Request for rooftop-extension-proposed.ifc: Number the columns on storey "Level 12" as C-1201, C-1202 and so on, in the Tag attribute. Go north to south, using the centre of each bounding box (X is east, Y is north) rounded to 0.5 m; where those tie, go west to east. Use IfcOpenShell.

First a look at what the model holds.

```python
import ifcopenshell
import ifcopenshell.util.element
import ifcopenshell.util.placement

model = ifcopenshell.open("rooftop-extension-proposed.ifc")
print(model.schema)
storey = next(s for s in model.by_type("IfcBuildingStorey") if s.Name == "Level 12")
columns = [e for e in ifcopenshell.util.element.get_decomposition(storey) if e.is_a("IfcColumn")]
for e in sorted(columns, key=lambda e: e.id()):
    origin = ifcopenshell.util.placement.get_local_placement(e.ObjectPlacement)[:3, 3]
    print(e.id(), e.Tag, e.Name, origin.round(2) + 0.0, sep=" | ")
```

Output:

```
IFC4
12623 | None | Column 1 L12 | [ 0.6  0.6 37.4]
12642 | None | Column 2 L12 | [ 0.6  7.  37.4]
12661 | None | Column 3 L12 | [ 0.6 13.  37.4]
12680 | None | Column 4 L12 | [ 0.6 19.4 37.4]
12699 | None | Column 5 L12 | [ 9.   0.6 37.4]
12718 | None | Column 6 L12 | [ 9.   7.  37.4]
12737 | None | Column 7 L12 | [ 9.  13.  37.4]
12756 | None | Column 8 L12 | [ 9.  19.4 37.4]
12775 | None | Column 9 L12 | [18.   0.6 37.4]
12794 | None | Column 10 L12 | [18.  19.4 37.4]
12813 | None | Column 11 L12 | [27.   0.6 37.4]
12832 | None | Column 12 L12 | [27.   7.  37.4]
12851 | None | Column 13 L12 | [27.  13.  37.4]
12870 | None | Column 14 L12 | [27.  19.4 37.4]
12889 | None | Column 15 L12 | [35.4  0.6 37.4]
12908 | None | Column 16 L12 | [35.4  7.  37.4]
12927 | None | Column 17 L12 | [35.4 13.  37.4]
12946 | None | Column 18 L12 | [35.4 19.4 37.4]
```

```python
import ifcopenshell
import ifcopenshell.geom
import ifcopenshell.util.element
import ifcopenshell.util.shape

model = ifcopenshell.open("rooftop-extension-proposed.ifc")
settings = ifcopenshell.geom.settings()
settings.set("use-world-coords", True)


def centre(element):
    shape = ifcopenshell.geom.create_shape(settings, element)
    return ifcopenshell.util.shape.get_bbox_centroid(shape.geometry)


storey = next(s for s in model.by_type("IfcBuildingStorey") if s.Name == "Level 12")
columns = [e for e in ifcopenshell.util.element.get_decomposition(storey) if e.is_a("IfcColumn")]

# Insertion points can sit at a corner or the storey origin, so sort by the geometry (in metres).
centres = {e: centre(e) for e in columns}
columns.sort(key=lambda e: (-round(centres[e][1] / 0.5), centres[e][0]))

for i, e in enumerate(columns, start=1):
    number = f"C-12{i:02d}"
    e.Tag = number
    print(e.id(), number)

model.write("rooftop-extension-proposed_edited.ifc")
```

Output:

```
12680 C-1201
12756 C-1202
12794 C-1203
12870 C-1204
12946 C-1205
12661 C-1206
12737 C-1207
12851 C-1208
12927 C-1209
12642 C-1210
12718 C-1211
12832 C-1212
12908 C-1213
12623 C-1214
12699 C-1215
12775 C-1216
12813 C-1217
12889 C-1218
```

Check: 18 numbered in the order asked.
